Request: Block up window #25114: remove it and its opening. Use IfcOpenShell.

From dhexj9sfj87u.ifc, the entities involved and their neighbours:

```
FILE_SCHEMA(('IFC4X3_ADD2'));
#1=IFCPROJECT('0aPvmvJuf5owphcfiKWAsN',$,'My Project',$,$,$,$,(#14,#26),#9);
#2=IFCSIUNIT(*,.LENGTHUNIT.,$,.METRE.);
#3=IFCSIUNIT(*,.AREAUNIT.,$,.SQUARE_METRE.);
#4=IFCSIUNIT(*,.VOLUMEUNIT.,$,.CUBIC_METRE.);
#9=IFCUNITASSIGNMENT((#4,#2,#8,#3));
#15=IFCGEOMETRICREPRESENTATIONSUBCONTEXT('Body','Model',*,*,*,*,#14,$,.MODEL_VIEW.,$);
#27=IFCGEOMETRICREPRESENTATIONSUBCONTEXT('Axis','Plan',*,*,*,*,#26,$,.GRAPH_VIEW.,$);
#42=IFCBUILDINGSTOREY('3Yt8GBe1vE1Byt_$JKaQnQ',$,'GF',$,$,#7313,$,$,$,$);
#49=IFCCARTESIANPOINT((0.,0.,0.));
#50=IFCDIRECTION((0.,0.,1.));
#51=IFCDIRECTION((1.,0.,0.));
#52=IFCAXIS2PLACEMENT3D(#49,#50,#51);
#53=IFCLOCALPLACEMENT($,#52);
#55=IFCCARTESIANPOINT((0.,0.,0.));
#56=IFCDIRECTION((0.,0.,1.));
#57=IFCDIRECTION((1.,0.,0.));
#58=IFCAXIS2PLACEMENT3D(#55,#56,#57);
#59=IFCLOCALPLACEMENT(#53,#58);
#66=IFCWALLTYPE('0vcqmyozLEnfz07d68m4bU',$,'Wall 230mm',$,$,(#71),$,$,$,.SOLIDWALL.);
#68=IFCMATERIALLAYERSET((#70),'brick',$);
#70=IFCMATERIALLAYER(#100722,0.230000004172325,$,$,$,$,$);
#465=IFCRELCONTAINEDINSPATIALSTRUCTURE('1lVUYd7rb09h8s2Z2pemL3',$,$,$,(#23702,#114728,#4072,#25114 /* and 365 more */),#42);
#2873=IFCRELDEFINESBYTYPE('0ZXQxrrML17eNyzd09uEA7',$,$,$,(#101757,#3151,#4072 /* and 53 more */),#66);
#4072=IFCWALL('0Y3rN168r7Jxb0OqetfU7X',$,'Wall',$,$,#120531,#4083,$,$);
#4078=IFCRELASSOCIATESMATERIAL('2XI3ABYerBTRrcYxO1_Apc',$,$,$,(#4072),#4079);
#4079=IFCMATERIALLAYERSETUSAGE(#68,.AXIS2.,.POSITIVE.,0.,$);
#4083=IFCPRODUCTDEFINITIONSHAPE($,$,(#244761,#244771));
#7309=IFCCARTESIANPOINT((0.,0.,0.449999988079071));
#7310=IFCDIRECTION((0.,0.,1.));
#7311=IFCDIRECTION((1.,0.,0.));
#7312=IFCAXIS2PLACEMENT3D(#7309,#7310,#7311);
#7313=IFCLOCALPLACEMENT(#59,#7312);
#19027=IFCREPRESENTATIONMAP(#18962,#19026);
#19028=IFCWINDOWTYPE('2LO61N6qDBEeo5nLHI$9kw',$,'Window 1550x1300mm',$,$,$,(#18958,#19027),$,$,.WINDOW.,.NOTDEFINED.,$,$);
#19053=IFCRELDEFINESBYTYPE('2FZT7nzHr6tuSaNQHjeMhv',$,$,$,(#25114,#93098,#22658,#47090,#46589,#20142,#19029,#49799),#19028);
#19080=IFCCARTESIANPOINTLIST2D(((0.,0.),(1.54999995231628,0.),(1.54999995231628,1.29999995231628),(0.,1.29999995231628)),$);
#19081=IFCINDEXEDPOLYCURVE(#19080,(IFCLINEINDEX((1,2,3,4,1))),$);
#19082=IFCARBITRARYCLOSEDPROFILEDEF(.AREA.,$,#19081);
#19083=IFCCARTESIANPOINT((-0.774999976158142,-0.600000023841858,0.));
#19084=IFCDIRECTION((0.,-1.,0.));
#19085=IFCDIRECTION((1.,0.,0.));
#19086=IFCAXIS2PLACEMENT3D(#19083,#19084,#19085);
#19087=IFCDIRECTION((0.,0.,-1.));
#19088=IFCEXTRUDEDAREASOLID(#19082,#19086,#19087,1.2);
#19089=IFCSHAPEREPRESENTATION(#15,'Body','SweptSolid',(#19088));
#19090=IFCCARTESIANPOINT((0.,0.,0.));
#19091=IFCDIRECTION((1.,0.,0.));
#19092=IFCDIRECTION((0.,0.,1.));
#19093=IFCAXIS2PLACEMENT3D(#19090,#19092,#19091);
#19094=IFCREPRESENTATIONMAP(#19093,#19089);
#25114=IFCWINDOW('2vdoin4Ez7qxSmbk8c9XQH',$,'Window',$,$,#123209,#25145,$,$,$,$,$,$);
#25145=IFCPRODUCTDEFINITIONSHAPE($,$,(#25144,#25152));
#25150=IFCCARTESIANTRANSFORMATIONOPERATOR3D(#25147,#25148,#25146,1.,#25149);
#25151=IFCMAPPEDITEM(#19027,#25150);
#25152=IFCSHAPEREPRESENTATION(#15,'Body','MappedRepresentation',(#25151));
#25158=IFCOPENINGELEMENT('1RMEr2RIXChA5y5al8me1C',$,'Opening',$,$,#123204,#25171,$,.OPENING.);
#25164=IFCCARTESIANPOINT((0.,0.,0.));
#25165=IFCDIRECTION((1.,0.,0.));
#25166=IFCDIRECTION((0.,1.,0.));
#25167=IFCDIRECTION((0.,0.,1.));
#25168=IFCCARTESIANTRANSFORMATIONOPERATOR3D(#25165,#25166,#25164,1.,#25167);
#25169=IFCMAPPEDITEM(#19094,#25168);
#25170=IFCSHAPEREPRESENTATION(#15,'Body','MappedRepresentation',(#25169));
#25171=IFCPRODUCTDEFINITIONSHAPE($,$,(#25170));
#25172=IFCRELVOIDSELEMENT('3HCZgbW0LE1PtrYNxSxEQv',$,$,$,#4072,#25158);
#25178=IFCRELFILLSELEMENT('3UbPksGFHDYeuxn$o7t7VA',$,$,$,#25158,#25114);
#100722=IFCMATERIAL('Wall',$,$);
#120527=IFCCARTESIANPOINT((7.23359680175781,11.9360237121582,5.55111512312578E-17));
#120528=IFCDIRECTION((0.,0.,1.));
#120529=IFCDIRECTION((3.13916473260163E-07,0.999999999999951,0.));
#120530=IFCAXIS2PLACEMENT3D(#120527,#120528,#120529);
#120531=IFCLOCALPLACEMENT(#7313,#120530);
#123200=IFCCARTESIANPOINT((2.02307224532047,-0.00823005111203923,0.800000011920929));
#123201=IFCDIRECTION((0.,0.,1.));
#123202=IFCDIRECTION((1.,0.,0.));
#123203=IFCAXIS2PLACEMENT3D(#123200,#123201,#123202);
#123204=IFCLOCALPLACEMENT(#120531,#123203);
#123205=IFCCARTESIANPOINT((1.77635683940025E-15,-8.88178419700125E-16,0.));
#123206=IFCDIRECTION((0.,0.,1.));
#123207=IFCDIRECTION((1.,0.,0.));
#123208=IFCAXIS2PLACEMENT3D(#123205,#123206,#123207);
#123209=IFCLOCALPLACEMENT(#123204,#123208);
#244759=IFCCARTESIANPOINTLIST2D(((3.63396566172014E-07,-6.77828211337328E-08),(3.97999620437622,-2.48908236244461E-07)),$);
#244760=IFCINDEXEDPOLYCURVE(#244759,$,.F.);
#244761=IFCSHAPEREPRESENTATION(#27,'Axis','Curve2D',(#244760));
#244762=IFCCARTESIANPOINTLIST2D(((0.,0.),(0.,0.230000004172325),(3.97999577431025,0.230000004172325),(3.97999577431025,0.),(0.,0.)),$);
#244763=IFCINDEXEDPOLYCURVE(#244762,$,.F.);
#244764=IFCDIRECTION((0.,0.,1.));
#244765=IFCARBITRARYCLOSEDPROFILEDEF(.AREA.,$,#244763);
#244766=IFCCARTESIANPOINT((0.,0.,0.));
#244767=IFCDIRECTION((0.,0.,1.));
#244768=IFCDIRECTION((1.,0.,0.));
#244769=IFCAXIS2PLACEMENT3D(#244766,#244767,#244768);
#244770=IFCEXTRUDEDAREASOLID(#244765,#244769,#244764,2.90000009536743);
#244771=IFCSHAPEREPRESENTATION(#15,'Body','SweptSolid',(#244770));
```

```python
import ifcopenshell
import ifcopenshell.api.feature
import ifcopenshell.api.root
import ifcopenshell.geom
import ifcopenshell.util.shape

model = ifcopenshell.open("dhexj9sfj87u.ifc")
settings = ifcopenshell.geom.settings()


def volume(element):
    """Net volume in cubic metres, openings subtracted."""
    shape = ifcopenshell.geom.create_shape(settings, element)
    return ifcopenshell.util.shape.get_volume(shape.geometry)


window = model.by_guid("2vdoin4Ez7qxSmbk8c9XQH")
opening = window.FillsVoids[0].RelatingOpeningElement
wall = opening.VoidsElements[0].RelatingBuildingElement
before = volume(wall)

ifcopenshell.api.root.remove_product(model, product=window)
ifcopenshell.api.feature.remove_feature(model, feature=opening)

after = volume(wall)

print(f"wall volume {before:.3f} -> {after:.3f} m3")

model.write("dhexj9sfj87u-out.ifc")
```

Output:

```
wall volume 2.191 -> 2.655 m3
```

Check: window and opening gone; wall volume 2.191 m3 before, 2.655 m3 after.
